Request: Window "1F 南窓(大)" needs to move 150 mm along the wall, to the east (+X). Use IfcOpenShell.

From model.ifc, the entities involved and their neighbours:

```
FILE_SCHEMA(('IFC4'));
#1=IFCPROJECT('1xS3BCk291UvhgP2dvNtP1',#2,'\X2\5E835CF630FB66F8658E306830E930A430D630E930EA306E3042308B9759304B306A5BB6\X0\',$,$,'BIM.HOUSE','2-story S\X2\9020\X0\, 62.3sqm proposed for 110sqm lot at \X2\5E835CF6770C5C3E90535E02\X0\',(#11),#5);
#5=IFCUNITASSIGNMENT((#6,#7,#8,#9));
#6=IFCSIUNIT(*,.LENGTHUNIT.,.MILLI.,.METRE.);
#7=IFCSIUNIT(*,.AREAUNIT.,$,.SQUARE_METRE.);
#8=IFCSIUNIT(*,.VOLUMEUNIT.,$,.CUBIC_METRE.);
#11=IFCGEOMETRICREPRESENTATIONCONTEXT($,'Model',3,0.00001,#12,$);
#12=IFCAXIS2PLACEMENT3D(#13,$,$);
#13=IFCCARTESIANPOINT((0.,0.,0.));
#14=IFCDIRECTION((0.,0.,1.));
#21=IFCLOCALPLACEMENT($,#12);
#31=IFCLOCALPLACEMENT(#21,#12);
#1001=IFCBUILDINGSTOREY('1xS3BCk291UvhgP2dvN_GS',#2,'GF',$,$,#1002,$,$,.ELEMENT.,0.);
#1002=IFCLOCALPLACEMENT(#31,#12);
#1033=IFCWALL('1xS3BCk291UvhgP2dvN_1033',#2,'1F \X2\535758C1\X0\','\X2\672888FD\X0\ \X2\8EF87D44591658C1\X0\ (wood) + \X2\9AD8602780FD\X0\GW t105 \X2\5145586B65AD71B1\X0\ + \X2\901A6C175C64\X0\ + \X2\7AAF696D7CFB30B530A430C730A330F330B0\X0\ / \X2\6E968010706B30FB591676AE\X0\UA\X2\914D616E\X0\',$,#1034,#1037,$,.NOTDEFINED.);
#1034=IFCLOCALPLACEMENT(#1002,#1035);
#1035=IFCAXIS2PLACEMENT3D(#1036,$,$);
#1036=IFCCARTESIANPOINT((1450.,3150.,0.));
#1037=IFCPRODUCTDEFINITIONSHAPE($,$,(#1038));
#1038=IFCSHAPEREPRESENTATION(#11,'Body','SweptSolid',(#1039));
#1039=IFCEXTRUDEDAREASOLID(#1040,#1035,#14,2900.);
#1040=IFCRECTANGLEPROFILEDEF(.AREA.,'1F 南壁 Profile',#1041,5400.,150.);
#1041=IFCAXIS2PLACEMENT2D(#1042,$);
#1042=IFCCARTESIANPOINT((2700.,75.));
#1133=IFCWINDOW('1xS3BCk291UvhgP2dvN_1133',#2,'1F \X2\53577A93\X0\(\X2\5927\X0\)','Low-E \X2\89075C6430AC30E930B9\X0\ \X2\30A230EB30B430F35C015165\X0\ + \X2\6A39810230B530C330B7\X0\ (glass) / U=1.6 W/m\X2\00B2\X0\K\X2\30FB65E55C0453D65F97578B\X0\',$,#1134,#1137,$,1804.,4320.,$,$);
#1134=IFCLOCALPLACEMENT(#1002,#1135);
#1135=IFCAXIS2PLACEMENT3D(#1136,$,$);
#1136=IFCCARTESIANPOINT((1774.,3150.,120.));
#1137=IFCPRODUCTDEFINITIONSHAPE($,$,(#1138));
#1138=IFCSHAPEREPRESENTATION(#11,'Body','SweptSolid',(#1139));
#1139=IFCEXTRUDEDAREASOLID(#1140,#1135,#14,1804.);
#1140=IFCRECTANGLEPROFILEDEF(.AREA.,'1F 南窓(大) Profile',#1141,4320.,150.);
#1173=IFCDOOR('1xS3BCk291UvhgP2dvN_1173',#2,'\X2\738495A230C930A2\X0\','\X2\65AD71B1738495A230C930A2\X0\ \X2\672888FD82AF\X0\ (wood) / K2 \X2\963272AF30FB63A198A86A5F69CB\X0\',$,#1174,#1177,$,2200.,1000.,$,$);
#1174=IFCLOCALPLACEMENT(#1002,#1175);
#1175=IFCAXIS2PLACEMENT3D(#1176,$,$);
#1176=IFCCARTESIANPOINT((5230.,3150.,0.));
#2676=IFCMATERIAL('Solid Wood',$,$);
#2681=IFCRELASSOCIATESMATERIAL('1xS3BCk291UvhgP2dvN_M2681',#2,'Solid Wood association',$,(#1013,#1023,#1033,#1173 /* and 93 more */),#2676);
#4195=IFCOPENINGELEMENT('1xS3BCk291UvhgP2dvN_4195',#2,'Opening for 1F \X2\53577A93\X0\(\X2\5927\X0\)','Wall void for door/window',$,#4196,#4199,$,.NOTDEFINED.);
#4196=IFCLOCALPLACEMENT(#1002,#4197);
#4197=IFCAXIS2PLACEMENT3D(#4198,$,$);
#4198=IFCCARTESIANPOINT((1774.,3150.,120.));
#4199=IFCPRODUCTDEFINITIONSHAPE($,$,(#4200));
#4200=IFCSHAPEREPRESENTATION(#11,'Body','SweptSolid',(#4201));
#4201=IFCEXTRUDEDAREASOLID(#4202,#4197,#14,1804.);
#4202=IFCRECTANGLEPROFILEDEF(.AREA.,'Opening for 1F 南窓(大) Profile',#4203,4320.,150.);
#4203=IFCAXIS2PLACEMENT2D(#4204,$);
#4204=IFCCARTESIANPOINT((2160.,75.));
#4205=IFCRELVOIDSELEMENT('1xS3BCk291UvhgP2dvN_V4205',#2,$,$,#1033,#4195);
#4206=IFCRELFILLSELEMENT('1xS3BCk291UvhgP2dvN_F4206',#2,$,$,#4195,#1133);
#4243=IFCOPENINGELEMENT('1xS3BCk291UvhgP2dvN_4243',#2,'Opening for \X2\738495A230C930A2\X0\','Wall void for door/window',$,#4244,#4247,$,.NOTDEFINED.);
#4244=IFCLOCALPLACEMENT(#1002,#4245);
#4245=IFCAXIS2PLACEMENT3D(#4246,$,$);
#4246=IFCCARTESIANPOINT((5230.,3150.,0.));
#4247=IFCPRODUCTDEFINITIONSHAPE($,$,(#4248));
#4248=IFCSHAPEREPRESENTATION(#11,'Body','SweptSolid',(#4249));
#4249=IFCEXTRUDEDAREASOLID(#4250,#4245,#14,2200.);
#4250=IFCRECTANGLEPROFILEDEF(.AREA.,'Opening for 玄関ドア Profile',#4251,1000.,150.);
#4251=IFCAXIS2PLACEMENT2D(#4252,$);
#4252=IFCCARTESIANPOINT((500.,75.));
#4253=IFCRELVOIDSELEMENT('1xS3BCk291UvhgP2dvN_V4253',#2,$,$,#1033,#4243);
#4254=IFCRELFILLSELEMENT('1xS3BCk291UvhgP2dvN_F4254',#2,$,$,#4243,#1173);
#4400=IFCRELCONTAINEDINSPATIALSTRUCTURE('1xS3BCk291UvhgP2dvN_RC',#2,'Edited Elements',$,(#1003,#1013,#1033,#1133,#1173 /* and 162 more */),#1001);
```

```python
import ifcopenshell
import ifcopenshell.api.geometry
import ifcopenshell.util.placement
import ifcopenshell.util.unit

model = ifcopenshell.open("model.ifc")
unit_scale = ifcopenshell.util.unit.calculate_unit_scale(model)

window = model.by_guid("1xS3BCk291UvhgP2dvN_1133")
opening = window.FillsVoids[0].RelatingOpeningElement
wall = opening.VoidsElements[0].RelatingBuildingElement

wall_matrix = ifcopenshell.util.placement.get_local_placement(wall.ObjectPlacement)
shift = wall_matrix[:3, 0] * 0.15 / unit_scale
before = ifcopenshell.util.placement.get_local_placement(window.ObjectPlacement)[:3, 3].copy()

# The window is not placed relative to its opening, so move both.
for product in (opening, window):
    matrix = ifcopenshell.util.placement.get_local_placement(product.ObjectPlacement)
    matrix[:3, 3] += shift
    ifcopenshell.api.geometry.edit_object_placement(model, product=product, matrix=matrix, is_si=False)

after = ifcopenshell.util.placement.get_local_placement(window.ObjectPlacement)[:3, 3]
print("window moved by", (after - before).round(3) + 0.0)

model.write("model-out.ifc")
```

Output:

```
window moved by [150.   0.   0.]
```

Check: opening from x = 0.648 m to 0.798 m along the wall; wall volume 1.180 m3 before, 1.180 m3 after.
